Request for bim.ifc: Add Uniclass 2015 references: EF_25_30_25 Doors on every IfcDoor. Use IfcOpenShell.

First a look at what the model holds.

```python
import ifcopenshell

model = ifcopenshell.open("bim.ifc")
print(model.schema)
print("classifications:", [c.Name for c in model.by_type("IfcClassification")])
for ifc_class in ("IfcDoor", "IfcRoof", "IfcStair", "IfcWall", "IfcWindow"):
    print(ifc_class, len(model.by_type(ifc_class)))
```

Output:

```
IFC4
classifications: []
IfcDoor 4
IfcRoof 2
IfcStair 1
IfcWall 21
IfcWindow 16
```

```python
import ifcopenshell
import ifcopenshell.api.classification

model = ifcopenshell.open("bim.ifc")

system = ifcopenshell.api.classification.add_classification(model, classification="Uniclass 2015")

codes = {
    "IfcDoor": ("EF_25_30_25", "Doors"),
}
for ifc_class, (code, name) in codes.items():
    products = model.by_type(ifc_class)
    ifcopenshell.api.classification.add_reference(
        model, products=products, classification=system, identification=code, name=name
    )
    print(code, len(products))

model.write("bim_rev.ifc")
```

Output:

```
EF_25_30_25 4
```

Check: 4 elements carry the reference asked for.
